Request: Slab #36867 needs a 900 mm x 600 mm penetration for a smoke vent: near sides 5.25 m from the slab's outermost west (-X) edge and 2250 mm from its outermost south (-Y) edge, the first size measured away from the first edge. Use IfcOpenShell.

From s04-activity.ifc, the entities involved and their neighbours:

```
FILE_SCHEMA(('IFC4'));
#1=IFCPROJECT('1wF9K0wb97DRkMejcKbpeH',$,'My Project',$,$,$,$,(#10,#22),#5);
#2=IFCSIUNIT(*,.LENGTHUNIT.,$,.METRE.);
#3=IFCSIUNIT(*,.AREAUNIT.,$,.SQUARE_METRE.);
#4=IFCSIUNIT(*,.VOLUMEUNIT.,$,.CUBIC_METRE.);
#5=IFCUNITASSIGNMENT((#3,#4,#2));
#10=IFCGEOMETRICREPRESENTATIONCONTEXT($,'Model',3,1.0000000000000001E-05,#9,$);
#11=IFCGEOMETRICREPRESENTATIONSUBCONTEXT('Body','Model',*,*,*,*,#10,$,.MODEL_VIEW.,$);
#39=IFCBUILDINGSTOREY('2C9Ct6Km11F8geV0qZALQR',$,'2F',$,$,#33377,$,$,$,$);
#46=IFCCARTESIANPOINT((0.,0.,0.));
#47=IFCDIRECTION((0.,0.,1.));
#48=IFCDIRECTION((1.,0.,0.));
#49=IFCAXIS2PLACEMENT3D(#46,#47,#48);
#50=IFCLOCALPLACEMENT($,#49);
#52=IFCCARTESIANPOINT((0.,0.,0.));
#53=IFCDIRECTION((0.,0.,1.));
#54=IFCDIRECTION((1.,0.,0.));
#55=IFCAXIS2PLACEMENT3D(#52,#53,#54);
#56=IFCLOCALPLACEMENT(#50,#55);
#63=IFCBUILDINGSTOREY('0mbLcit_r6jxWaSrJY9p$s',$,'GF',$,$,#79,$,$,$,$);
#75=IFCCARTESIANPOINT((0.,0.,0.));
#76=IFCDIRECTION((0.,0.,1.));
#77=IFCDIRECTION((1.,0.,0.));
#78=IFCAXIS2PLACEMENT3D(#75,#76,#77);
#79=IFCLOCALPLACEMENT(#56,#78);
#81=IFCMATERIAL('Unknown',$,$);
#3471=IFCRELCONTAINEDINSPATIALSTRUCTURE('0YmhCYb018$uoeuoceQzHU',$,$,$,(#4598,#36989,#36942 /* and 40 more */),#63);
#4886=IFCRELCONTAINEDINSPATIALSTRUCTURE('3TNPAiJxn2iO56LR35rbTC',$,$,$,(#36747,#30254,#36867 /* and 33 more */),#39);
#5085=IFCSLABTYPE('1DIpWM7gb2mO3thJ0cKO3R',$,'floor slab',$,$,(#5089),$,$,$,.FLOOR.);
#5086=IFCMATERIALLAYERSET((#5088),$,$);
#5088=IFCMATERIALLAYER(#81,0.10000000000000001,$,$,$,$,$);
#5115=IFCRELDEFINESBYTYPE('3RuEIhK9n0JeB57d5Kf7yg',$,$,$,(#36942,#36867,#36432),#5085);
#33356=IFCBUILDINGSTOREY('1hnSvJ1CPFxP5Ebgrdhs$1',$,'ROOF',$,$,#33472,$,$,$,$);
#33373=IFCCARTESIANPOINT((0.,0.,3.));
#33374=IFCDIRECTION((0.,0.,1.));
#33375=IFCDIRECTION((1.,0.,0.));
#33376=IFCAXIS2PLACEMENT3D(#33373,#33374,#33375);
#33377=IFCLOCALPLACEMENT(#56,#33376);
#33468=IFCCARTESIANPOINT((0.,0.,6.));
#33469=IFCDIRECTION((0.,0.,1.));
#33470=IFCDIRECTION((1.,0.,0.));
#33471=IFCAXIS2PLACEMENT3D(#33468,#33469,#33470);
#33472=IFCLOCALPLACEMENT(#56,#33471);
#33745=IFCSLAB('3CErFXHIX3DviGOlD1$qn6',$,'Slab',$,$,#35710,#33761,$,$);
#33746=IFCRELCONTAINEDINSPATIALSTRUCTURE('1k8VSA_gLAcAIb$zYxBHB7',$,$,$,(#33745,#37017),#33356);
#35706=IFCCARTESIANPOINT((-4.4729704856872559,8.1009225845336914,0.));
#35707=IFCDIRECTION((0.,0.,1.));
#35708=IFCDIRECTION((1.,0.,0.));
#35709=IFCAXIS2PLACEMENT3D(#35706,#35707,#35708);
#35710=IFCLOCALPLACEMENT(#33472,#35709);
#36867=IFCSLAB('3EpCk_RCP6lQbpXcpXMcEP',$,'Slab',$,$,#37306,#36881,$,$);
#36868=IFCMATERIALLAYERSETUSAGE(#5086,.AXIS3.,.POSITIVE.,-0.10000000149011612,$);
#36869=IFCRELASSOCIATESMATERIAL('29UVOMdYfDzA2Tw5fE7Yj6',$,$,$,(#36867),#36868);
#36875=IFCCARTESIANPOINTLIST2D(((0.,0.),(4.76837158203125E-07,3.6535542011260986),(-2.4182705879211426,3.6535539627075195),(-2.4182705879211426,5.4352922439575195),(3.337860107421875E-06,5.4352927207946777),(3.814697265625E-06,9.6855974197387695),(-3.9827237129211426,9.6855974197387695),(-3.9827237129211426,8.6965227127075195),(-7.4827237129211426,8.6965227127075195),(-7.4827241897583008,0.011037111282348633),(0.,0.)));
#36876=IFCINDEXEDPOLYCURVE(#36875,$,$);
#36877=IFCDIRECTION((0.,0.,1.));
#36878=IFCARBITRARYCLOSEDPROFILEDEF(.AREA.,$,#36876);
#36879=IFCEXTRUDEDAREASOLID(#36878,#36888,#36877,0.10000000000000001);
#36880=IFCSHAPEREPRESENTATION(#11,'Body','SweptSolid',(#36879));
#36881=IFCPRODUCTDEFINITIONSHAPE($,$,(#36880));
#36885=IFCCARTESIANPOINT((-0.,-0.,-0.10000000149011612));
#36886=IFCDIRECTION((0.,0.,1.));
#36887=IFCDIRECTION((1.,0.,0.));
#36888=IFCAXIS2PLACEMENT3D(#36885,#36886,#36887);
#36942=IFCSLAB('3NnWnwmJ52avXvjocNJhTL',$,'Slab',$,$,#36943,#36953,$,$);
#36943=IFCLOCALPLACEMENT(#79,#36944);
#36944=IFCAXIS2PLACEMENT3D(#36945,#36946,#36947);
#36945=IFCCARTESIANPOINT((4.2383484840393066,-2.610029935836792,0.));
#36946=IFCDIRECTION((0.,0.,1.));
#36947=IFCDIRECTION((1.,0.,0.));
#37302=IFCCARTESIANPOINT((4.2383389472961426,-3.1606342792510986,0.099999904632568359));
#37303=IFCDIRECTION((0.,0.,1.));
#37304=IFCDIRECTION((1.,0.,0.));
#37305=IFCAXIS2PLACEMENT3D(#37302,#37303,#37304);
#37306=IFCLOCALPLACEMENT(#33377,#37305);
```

```python
import numpy as np
import ifcopenshell
import ifcopenshell.api.feature
import ifcopenshell.api.geometry
import ifcopenshell.api.root
import ifcopenshell.geom
import ifcopenshell.util.placement
import ifcopenshell.util.representation
import ifcopenshell.util.shape
import ifcopenshell.util.unit

model = ifcopenshell.open("s04-activity.ifc")
unit_scale = ifcopenshell.util.unit.calculate_unit_scale(model)
settings = ifcopenshell.geom.settings()


def volume(element):
    """Net volume in cubic metres, openings subtracted."""
    shape = ifcopenshell.geom.create_shape(settings, element)
    return ifcopenshell.util.shape.get_volume(shape.geometry)


slab = model.by_guid("3EpCk_RCP6lQbpXcpXMcEP")
before = volume(slab)

# Extent in the slab's own axes, in metres. The edges named are its -X and -Y sides.
slab_shape = ifcopenshell.geom.create_shape(settings, slab)
vertices = ifcopenshell.util.shape.get_vertices(slab_shape.geometry)
x_min, y_min, bottom = vertices.min(axis=0)
top = vertices[:, 2].max()

opening = ifcopenshell.api.root.create_entity(model, ifc_class="IfcOpeningElement", name="Smoke vent opening", predefined_type="OPENING")
context = ifcopenshell.util.representation.get_context(model, "Model", "Body", "MODEL_VIEW")
width, depth = 0.9, 0.6
outline = [(0.0, 0.0), (width, 0.0), (width, depth), (0.0, depth), (0.0, 0.0)]
# Overshoot both faces by 50 mm so the cut is clean.
shape = ifcopenshell.api.geometry.add_slab_representation(
    model, context=context, depth=top - bottom + 0.1, polyline=outline
)
ifcopenshell.api.geometry.assign_representation(model, product=opening, representation=shape)

matrix = ifcopenshell.util.placement.get_local_placement(slab.ObjectPlacement)
matrix[:, 3] = matrix @ np.append(np.array([x_min + 5.25, y_min + 2.25, bottom - 0.05]) / unit_scale, 1.0)
ifcopenshell.api.geometry.edit_object_placement(model, product=opening, matrix=matrix, is_si=False)
ifcopenshell.api.feature.add_feature(model, feature=opening, element=slab)

after = volume(slab)

print(f"slab volume {before:.3f} -> {after:.3f} m3")

model.write("s04-activity-out.ifc")
```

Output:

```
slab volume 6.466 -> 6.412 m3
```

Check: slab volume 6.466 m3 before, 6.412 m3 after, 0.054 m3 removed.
